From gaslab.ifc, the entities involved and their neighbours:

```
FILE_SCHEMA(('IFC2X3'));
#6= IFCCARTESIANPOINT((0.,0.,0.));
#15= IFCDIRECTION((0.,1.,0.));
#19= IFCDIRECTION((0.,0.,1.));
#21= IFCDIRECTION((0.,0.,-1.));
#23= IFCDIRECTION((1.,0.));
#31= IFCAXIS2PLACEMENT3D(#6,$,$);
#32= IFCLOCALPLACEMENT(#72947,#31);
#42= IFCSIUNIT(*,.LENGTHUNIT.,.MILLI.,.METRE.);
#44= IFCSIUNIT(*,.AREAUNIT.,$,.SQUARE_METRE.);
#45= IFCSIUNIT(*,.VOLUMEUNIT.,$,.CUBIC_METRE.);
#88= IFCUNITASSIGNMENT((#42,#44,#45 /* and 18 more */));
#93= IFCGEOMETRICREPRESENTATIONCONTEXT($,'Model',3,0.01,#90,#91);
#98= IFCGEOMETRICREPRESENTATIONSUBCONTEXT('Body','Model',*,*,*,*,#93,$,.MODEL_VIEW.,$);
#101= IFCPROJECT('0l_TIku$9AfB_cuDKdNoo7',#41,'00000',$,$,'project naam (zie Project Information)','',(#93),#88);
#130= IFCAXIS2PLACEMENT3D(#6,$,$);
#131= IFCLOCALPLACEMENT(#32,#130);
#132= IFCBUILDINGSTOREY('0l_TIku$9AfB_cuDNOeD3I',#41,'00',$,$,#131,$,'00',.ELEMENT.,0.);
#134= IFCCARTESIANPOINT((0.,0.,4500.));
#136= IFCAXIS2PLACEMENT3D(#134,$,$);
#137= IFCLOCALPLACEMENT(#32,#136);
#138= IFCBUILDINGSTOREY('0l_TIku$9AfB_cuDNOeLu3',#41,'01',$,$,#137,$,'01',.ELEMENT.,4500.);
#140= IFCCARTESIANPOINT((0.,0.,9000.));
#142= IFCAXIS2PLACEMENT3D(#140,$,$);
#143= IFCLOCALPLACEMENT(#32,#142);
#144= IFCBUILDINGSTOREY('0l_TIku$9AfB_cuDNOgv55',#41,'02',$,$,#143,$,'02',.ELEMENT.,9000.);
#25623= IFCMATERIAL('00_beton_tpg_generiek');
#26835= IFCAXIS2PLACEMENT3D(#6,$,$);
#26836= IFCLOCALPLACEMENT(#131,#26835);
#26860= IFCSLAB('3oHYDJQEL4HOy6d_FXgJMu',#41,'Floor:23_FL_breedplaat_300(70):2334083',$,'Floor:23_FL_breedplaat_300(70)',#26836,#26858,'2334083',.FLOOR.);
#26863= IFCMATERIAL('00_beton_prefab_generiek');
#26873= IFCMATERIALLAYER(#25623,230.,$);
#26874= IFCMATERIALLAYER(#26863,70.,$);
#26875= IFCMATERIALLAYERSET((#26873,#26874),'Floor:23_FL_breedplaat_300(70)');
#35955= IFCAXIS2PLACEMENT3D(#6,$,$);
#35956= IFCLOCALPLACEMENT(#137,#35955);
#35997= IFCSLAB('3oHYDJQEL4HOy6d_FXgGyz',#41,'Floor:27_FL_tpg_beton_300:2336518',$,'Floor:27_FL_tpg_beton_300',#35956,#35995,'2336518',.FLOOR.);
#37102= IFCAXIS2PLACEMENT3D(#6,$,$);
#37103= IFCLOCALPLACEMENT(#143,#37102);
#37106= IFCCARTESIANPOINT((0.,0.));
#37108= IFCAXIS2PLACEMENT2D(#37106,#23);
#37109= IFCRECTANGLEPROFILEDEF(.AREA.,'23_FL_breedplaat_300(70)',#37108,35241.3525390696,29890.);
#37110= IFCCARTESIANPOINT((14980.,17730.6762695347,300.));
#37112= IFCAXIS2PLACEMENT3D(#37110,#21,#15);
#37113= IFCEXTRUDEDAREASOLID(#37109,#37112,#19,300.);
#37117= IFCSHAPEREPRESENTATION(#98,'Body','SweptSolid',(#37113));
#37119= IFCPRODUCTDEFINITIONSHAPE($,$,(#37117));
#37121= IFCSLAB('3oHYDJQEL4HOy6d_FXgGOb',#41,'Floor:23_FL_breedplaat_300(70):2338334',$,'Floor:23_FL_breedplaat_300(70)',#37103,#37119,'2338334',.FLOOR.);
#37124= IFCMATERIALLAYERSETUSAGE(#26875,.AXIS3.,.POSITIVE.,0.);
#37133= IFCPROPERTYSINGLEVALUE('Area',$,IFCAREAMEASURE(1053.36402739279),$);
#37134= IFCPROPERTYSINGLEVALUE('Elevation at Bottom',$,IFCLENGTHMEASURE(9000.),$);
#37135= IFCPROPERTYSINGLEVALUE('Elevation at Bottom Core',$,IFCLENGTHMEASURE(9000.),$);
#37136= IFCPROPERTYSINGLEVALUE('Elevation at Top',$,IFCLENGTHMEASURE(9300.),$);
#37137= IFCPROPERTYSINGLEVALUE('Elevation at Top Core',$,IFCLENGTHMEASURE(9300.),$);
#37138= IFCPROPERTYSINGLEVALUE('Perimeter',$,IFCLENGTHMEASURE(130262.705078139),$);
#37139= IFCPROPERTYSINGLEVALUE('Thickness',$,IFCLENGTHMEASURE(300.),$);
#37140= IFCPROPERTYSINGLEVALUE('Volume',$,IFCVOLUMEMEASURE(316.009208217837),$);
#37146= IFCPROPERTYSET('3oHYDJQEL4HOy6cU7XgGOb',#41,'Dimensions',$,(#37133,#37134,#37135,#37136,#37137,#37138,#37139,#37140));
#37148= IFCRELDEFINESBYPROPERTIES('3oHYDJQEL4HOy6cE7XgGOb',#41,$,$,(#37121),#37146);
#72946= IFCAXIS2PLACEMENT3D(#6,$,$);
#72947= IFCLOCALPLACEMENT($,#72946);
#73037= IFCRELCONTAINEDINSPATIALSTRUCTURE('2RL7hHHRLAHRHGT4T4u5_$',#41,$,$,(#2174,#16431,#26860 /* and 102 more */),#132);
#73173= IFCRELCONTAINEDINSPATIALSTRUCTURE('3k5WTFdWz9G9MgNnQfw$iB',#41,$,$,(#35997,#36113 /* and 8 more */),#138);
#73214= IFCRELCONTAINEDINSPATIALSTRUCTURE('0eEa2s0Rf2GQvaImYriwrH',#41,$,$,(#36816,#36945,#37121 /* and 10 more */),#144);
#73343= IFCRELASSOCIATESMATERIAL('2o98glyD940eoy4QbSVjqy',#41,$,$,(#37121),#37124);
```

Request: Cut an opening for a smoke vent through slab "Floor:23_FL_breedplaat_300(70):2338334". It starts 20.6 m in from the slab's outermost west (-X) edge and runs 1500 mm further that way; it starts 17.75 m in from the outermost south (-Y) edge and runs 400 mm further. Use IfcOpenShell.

```python
import numpy as np
import ifcopenshell
import ifcopenshell.api.feature
import ifcopenshell.api.geometry
import ifcopenshell.api.pset
import ifcopenshell.api.root
import ifcopenshell.geom
import ifcopenshell.util.element
import ifcopenshell.util.placement
import ifcopenshell.util.representation
import ifcopenshell.util.shape
import ifcopenshell.util.unit

model = ifcopenshell.open("gaslab.ifc")
unit_scale = ifcopenshell.util.unit.calculate_unit_scale(model)
area_scale = ifcopenshell.util.unit.calculate_unit_scale(model, "AREAUNIT")
volume_scale = ifcopenshell.util.unit.calculate_unit_scale(model, "VOLUMEUNIT")
settings = ifcopenshell.geom.settings()


def volume(element):
    """Net volume in cubic metres, openings subtracted."""
    shape = ifcopenshell.geom.create_shape(settings, element)
    return ifcopenshell.util.shape.get_volume(shape.geometry)


slab = model.by_id(37121)
before = volume(slab)

# Extent in the slab's own axes, in metres. The edges named are its -X and -Y sides.
slab_shape = ifcopenshell.geom.create_shape(settings, slab)
vertices = ifcopenshell.util.shape.get_vertices(slab_shape.geometry)
x_min, y_min, bottom = vertices.min(axis=0)
top = vertices[:, 2].max()

opening = ifcopenshell.api.root.create_entity(model, ifc_class="IfcOpeningElement", name="Smoke vent opening")
context = ifcopenshell.util.representation.get_context(model, "Model", "Body", "MODEL_VIEW")
width, depth = 1.5, 0.4
outline = [(0.0, 0.0), (width, 0.0), (width, depth), (0.0, depth), (0.0, 0.0)]
# Overshoot both faces by 50 mm so the cut is clean.
shape = ifcopenshell.api.geometry.add_slab_representation(
    model, context=context, depth=top - bottom + 0.1, polyline=outline
)
ifcopenshell.api.geometry.assign_representation(model, product=opening, representation=shape)

matrix = ifcopenshell.util.placement.get_local_placement(slab.ObjectPlacement)
matrix[:, 3] = matrix @ np.append(np.array([x_min + 20.6, y_min + 17.75, bottom - 0.05]) / unit_scale, 1.0)
ifcopenshell.api.geometry.edit_object_placement(model, product=opening, matrix=matrix, is_si=False)
ifcopenshell.api.feature.add_feature(model, feature=opening, element=slab)

after = volume(slab)

# Update the slab's stored quantities.
pset = model.by_id(ifcopenshell.util.element.get_pset(slab, "Dimensions", should_inherit=False)["id"])
ifcopenshell.api.pset.edit_pset(model, pset=pset, properties={
    "Area": model.create_entity("IfcAreaMeasure", after / (top - bottom) / area_scale),
    "Volume": model.create_entity("IfcVolumeMeasure", after / volume_scale),
})

print(f"slab volume {before:.3f} -> {after:.3f} m3")

model.write("gaslab-out.ifc")
```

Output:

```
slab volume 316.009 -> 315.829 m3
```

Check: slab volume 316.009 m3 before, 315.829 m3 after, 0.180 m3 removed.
